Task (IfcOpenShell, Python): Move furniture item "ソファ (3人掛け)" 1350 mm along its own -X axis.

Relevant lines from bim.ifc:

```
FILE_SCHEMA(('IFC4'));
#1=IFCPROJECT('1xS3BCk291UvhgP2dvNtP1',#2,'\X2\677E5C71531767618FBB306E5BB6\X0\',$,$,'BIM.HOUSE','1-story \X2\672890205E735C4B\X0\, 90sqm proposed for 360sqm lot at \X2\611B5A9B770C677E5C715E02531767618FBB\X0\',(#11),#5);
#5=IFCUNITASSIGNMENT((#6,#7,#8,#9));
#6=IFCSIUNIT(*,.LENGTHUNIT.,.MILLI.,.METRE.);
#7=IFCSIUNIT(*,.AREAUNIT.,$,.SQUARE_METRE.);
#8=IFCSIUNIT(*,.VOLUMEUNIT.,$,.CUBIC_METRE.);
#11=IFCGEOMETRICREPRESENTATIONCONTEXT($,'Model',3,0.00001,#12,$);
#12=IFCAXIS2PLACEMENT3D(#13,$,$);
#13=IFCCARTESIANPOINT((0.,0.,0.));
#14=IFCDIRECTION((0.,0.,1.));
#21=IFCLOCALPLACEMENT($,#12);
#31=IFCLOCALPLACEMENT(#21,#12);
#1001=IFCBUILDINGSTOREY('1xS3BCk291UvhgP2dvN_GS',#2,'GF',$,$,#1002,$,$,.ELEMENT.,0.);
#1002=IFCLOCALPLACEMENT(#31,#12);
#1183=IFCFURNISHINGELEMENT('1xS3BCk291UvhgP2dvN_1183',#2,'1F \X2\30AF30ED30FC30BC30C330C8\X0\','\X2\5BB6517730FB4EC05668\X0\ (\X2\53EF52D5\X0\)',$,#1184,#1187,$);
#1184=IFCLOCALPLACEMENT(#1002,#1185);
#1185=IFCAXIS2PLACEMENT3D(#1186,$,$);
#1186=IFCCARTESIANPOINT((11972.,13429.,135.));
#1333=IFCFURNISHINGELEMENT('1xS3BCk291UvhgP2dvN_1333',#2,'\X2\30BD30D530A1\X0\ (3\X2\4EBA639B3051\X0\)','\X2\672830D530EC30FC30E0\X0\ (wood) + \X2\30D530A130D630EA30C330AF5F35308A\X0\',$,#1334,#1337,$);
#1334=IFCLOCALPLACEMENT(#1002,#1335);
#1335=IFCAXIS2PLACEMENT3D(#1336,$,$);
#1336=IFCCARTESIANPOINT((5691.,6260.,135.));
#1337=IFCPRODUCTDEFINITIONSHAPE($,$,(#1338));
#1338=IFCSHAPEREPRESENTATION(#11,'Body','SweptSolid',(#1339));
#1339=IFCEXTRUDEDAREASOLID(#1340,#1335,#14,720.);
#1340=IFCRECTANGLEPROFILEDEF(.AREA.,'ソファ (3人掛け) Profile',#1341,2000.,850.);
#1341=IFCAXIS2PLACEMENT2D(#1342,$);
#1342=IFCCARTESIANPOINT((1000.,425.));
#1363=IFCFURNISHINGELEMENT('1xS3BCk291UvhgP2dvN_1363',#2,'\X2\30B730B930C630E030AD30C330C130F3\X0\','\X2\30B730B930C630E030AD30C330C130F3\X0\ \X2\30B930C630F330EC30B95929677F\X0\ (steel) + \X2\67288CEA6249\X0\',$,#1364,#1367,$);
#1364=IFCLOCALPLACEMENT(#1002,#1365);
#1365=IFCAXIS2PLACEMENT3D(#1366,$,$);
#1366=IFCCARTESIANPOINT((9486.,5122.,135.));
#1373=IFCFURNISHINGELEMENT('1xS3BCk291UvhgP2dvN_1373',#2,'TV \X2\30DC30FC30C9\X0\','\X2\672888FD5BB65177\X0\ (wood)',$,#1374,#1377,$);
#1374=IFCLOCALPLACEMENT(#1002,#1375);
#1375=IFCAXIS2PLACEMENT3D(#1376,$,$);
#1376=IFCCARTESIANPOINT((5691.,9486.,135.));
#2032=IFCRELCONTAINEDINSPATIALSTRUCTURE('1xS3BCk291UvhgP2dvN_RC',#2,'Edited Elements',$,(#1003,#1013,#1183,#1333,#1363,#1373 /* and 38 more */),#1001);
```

```python
import ifcopenshell
import ifcopenshell.api.geometry
import ifcopenshell.util.placement

model = ifcopenshell.open("bim.ifc")

item = model.by_id(1333)
matrix = ifcopenshell.util.placement.get_local_placement(item.ObjectPlacement)
matrix[:3, 3] -= matrix[:3, 0] * 1350.0
ifcopenshell.api.geometry.edit_object_placement(model, product=item, matrix=matrix, is_si=False)

print(ifcopenshell.util.placement.get_local_placement(item.ObjectPlacement).round(3) + 0.0)

model.write("bim_v2.ifc")
```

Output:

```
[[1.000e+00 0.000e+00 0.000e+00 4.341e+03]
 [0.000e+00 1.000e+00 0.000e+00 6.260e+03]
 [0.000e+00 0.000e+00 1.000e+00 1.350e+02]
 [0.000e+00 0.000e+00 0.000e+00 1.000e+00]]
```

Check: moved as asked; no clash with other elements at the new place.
